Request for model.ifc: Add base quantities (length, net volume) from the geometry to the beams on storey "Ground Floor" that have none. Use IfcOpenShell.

First a look at what the model holds.

```python
import ifcopenshell
import ifcopenshell.util.element
import ifcopenshell.util.unit

model = ifcopenshell.open("model.ifc")
print(model.schema)
for unit_type in ("LENGTHUNIT", "AREAUNIT", "VOLUMEUNIT"):
    print(unit_type, ifcopenshell.util.unit.calculate_unit_scale(model, unit_type))
storey = next(s for s in model.by_type("IfcBuildingStorey") if s.Name == "Ground Floor")
beams = [e for e in ifcopenshell.util.element.get_decomposition(storey) if e.is_a("IfcBeam")]
for e in sorted(beams, key=lambda e: e.id()):
    print(e.id(), e.is_a(), e.Name, list(ifcopenshell.util.element.get_psets(e, qtos_only=True)), sep=" | ")
```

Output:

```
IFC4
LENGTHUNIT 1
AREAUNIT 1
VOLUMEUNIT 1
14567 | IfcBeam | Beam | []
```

```python
import ifcopenshell
import ifcopenshell.api.pset
import ifcopenshell.geom
import ifcopenshell.util.element
import ifcopenshell.util.shape
import ifcopenshell.util.unit

model = ifcopenshell.open("model.ifc")
unit_scale = ifcopenshell.util.unit.calculate_unit_scale(model)
volume_scale = ifcopenshell.util.unit.calculate_unit_scale(model, "VOLUMEUNIT")
settings = ifcopenshell.geom.settings()

storey = next(s for s in model.by_type("IfcBuildingStorey") if s.Name == "Ground Floor")
beams = [e for e in ifcopenshell.util.element.get_decomposition(storey) if e.is_a("IfcBeam")]

for e in sorted(beams, key=lambda e: e.id()):
    if ifcopenshell.util.element.get_psets(e, qtos_only=True, should_inherit=False):
        continue
    # Geometry comes back in metres, in the element's own axes.
    shape = ifcopenshell.geom.create_shape(settings, e)
    values = {
        "Length": ifcopenshell.util.shape.get_max_xyz(shape.geometry) / unit_scale,
        "NetVolume": ifcopenshell.util.shape.get_volume(shape.geometry) / volume_scale,
    }
    qto = ifcopenshell.api.pset.add_qto(model, product=e, name="Qto_BeamBaseQuantities")
    ifcopenshell.api.pset.edit_qto(model, qto=qto, properties=values)
    print(e.id(), {k: round(v, 3) for k, v in values.items()})

model.write("model-out.ifc")
```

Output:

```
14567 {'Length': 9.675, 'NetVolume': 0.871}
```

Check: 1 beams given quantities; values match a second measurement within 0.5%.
